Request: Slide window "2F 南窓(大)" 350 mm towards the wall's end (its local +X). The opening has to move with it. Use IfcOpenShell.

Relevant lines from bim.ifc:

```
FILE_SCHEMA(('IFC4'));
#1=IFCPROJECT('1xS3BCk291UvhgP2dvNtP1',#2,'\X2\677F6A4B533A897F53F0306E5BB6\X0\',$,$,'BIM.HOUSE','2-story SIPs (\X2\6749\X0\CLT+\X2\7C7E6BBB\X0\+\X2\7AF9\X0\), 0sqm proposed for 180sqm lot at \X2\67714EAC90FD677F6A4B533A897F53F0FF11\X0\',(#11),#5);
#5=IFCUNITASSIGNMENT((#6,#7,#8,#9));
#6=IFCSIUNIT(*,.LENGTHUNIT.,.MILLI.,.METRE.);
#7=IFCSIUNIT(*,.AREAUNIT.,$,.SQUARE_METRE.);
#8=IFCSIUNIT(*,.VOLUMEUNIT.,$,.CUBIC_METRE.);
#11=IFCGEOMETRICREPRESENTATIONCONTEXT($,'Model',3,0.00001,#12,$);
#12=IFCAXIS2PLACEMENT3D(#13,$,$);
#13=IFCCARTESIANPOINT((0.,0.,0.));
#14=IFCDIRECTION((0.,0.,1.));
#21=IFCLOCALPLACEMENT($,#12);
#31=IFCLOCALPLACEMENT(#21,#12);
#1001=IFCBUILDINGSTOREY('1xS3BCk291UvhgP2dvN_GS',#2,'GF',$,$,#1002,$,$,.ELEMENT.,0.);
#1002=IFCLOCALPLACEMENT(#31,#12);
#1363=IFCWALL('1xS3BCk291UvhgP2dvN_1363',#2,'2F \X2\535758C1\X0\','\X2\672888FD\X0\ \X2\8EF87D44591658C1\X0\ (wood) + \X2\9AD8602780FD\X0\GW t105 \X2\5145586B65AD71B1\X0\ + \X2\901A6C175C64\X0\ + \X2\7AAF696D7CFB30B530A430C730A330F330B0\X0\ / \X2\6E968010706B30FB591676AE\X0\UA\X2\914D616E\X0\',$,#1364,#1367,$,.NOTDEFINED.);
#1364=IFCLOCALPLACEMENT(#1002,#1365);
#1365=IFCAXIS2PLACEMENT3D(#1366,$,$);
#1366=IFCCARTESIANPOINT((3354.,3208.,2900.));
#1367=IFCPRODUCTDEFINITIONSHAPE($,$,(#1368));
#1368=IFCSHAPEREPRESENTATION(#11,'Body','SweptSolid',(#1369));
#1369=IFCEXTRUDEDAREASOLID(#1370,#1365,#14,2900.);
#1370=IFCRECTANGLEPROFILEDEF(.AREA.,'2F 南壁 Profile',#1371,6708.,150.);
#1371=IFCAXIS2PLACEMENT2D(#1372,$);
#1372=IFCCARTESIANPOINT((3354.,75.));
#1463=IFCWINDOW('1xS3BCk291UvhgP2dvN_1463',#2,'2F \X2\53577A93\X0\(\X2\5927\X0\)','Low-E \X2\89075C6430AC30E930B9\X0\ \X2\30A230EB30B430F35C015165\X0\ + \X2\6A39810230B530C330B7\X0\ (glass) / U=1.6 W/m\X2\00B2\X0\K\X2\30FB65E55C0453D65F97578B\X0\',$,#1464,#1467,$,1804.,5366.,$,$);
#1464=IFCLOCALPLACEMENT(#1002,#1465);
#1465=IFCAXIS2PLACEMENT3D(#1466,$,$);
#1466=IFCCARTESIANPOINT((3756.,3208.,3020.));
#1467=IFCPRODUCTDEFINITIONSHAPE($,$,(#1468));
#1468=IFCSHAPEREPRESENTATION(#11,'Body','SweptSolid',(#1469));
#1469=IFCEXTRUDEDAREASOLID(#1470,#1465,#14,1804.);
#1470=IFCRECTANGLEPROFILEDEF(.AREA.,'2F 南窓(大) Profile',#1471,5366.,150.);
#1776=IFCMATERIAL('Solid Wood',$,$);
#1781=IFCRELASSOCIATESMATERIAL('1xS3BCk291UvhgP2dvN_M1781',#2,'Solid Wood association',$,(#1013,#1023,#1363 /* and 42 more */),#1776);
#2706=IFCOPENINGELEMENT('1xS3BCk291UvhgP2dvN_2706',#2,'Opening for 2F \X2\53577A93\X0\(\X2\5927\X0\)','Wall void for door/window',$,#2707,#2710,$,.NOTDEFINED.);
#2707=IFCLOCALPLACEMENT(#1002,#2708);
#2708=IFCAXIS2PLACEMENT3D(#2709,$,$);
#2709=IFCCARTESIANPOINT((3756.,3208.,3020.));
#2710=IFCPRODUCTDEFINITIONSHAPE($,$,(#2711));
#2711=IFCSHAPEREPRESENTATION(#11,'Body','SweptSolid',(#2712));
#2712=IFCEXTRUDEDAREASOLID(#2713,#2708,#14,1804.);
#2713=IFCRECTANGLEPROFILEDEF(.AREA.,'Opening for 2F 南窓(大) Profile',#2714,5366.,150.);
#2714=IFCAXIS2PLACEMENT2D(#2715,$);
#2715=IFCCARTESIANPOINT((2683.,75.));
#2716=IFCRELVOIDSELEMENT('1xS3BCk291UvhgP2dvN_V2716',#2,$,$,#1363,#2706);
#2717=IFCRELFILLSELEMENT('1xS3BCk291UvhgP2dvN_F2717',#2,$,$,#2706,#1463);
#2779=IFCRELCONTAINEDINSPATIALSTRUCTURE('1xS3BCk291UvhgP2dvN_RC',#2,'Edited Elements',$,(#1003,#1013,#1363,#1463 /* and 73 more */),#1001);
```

```python
import ifcopenshell
import ifcopenshell.api.geometry
import ifcopenshell.util.placement
import ifcopenshell.util.unit

model = ifcopenshell.open("bim.ifc")
unit_scale = ifcopenshell.util.unit.calculate_unit_scale(model)

window = model.by_id(1463)
opening = window.FillsVoids[0].RelatingOpeningElement
wall = opening.VoidsElements[0].RelatingBuildingElement

wall_matrix = ifcopenshell.util.placement.get_local_placement(wall.ObjectPlacement)
shift = wall_matrix[:3, 0] * 0.35 / unit_scale
before = ifcopenshell.util.placement.get_local_placement(window.ObjectPlacement)[:3, 3].copy()

# The window is not placed relative to its opening, so move both.
for product in (opening, window):
    matrix = ifcopenshell.util.placement.get_local_placement(product.ObjectPlacement)
    matrix[:3, 3] += shift
    ifcopenshell.api.geometry.edit_object_placement(model, product=product, matrix=matrix, is_si=False)

after = ifcopenshell.util.placement.get_local_placement(window.ObjectPlacement)[:3, 3]
print("window moved by", (after - before).round(3) + 0.0)

model.write("bim_updated.ifc")
```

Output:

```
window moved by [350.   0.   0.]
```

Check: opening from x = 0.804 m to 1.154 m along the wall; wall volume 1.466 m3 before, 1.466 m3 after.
